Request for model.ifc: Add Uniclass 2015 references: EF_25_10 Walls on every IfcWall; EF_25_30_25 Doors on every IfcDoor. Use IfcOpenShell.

First a look at what the model holds.

```python
import ifcopenshell

model = ifcopenshell.open("model.ifc")
print(model.schema)
print("classifications:", [c.Name for c in model.by_type("IfcClassification")])
for ifc_class in ("IfcDoor", "IfcRoof", "IfcStair", "IfcWall", "IfcWindow"):
    print(ifc_class, len(model.by_type(ifc_class)))
```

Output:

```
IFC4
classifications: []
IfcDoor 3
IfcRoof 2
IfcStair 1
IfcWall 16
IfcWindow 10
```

```python
import ifcopenshell
import ifcopenshell.api.classification

model = ifcopenshell.open("model.ifc")

system = ifcopenshell.api.classification.add_classification(model, classification="Uniclass 2015")

codes = {
    "IfcWall": ("EF_25_10", "Walls"),
    "IfcDoor": ("EF_25_30_25", "Doors"),
}
for ifc_class, (code, name) in codes.items():
    products = model.by_type(ifc_class)
    ifcopenshell.api.classification.add_reference(
        model, products=products, classification=system, identification=code, name=name
    )
    print(code, len(products))

model.write("model_v2.ifc")
```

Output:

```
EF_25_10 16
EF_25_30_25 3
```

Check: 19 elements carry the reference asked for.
